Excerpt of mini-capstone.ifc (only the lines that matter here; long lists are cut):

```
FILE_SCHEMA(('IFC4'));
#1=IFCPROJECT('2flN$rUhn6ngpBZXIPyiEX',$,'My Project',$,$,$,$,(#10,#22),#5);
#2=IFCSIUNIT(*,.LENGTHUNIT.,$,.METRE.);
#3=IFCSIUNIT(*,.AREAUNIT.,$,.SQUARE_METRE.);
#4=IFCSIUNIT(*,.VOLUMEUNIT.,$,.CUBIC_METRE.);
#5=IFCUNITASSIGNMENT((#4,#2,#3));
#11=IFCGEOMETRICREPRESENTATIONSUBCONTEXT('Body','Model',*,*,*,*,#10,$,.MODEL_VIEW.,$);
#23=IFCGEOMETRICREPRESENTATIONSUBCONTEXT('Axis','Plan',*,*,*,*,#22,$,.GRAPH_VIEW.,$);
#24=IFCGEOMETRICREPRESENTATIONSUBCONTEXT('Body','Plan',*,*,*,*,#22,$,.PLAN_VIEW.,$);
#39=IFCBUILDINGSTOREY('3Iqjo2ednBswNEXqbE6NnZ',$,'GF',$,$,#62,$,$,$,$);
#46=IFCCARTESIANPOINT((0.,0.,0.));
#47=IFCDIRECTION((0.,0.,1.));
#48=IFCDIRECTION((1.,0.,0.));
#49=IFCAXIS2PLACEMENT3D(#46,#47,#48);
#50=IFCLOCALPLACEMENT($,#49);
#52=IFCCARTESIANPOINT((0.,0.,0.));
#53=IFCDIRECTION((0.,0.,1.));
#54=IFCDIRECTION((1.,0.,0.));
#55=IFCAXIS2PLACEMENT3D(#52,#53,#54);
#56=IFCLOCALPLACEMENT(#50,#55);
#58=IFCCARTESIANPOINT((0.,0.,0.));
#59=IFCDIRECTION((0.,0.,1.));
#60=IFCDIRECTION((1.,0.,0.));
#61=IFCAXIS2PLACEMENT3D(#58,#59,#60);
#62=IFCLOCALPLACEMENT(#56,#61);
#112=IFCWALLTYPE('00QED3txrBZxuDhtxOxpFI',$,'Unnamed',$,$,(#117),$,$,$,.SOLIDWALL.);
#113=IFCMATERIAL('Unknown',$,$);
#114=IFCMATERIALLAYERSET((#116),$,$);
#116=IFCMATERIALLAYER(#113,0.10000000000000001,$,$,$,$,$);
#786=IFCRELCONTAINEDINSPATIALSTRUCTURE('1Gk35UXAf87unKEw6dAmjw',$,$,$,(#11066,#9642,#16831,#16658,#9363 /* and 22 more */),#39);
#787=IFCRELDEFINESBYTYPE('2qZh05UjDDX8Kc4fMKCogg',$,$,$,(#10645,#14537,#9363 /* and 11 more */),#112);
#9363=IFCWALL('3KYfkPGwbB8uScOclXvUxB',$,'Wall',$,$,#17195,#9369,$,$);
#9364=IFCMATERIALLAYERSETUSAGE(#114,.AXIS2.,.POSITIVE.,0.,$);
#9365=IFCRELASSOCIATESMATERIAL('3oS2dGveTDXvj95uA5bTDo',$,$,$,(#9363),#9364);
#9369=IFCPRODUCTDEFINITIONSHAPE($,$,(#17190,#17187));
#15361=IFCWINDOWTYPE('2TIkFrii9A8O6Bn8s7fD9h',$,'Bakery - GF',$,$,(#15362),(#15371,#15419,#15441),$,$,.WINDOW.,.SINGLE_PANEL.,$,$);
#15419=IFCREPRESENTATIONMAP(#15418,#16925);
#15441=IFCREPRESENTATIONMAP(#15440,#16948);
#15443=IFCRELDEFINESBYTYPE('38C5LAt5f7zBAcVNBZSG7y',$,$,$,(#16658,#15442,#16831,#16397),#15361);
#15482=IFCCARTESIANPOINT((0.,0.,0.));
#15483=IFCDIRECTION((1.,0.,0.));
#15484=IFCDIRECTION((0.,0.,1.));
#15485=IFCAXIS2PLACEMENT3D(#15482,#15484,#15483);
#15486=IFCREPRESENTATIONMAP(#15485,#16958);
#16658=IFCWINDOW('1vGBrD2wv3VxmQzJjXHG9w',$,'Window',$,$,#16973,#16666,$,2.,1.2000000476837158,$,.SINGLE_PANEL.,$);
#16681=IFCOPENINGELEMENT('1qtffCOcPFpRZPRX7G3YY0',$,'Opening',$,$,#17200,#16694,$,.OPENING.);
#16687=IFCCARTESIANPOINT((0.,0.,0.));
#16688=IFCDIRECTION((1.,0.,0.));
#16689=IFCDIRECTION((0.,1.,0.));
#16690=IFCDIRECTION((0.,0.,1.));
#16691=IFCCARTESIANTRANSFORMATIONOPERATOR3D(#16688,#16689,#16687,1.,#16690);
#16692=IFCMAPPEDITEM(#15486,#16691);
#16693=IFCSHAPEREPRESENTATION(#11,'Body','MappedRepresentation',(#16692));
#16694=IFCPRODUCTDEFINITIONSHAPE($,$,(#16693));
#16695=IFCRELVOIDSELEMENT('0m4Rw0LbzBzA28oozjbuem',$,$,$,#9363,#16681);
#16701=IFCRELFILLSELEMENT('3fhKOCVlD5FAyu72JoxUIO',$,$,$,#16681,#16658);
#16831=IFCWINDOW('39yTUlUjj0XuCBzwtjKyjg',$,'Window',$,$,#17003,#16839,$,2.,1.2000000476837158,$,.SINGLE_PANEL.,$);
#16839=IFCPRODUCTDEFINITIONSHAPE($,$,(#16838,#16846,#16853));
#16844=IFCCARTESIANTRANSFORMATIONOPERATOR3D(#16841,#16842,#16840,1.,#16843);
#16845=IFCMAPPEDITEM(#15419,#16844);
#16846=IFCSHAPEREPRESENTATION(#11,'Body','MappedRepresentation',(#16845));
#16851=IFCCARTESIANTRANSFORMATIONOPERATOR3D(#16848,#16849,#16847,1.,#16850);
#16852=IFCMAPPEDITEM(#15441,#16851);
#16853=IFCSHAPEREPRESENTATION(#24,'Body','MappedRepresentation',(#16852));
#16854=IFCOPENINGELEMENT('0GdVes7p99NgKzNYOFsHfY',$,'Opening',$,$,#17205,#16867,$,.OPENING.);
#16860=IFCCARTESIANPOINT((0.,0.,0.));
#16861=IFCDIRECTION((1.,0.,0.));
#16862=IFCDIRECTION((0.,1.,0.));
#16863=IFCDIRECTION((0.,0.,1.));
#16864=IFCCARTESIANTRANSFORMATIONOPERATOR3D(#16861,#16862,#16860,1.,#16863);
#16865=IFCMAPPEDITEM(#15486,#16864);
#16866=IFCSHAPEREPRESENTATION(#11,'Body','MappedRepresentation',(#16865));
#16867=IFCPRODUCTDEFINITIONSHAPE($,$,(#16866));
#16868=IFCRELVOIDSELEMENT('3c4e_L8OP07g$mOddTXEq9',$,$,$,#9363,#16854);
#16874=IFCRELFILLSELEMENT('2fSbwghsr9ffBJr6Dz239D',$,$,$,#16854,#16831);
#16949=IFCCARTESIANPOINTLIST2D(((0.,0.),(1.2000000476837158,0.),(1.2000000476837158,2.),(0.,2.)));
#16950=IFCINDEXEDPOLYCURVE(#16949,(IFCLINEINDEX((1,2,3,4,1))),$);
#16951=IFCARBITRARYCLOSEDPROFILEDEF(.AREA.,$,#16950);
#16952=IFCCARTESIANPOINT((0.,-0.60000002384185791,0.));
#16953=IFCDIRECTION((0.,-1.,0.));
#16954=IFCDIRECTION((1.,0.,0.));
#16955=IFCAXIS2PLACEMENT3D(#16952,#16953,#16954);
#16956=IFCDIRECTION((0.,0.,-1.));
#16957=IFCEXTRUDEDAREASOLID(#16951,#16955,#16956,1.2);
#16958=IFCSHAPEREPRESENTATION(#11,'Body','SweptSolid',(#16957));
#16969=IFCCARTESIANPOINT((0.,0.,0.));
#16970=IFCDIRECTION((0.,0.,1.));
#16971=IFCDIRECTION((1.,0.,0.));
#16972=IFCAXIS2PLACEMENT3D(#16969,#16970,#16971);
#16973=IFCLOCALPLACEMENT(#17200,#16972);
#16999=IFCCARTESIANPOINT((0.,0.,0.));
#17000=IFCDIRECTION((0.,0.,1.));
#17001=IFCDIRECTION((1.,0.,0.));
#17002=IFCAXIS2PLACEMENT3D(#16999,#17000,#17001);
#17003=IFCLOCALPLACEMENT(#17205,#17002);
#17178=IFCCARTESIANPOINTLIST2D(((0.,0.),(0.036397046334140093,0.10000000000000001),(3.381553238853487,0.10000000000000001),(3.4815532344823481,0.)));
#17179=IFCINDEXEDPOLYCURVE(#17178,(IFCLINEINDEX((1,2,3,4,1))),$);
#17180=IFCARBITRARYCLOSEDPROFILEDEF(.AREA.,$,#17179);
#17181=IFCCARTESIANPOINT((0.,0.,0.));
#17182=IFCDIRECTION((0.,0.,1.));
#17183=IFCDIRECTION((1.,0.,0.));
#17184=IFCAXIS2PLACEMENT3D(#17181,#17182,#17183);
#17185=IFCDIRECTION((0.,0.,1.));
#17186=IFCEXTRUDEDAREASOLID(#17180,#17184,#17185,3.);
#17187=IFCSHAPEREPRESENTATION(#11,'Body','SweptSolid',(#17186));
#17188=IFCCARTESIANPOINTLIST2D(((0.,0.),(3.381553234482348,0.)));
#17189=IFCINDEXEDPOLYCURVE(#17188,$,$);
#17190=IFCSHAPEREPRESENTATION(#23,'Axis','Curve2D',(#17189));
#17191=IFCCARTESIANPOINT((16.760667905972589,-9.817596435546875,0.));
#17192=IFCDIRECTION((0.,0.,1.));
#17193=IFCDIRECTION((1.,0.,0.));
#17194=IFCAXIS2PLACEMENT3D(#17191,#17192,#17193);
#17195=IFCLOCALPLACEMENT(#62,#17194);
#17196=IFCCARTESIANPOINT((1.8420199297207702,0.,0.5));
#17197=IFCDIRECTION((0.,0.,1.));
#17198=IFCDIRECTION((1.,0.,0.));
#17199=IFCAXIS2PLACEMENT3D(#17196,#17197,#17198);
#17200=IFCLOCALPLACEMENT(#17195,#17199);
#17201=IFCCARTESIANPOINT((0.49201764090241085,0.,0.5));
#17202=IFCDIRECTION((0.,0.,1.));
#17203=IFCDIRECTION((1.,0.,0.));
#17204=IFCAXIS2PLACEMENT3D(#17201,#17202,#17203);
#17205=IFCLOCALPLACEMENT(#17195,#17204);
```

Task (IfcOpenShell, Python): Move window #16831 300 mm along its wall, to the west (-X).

```python
import ifcopenshell
import ifcopenshell.api.geometry
import ifcopenshell.util.placement
import ifcopenshell.util.unit

model = ifcopenshell.open("mini-capstone.ifc")
unit_scale = ifcopenshell.util.unit.calculate_unit_scale(model)

window = model.by_guid("39yTUlUjj0XuCBzwtjKyjg")
opening = window.FillsVoids[0].RelatingOpeningElement
wall = opening.VoidsElements[0].RelatingBuildingElement

wall_matrix = ifcopenshell.util.placement.get_local_placement(wall.ObjectPlacement)
shift = wall_matrix[:3, 0] * -0.3 / unit_scale
before = ifcopenshell.util.placement.get_local_placement(window.ObjectPlacement)[:3, 3].copy()

# The window is placed relative to its opening, so it follows when the opening moves.
matrix = ifcopenshell.util.placement.get_local_placement(opening.ObjectPlacement)
matrix[:3, 3] += shift
ifcopenshell.api.geometry.edit_object_placement(
    model, product=opening, matrix=matrix, is_si=False, should_transform_children=True
)

after = ifcopenshell.util.placement.get_local_placement(window.ObjectPlacement)[:3, 3]
print("window moved by", (after - before).round(3) + 0.0)

model.write("mini-capstone_edited.ifc")
```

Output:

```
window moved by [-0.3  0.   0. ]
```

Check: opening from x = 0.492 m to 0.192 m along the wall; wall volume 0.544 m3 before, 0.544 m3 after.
